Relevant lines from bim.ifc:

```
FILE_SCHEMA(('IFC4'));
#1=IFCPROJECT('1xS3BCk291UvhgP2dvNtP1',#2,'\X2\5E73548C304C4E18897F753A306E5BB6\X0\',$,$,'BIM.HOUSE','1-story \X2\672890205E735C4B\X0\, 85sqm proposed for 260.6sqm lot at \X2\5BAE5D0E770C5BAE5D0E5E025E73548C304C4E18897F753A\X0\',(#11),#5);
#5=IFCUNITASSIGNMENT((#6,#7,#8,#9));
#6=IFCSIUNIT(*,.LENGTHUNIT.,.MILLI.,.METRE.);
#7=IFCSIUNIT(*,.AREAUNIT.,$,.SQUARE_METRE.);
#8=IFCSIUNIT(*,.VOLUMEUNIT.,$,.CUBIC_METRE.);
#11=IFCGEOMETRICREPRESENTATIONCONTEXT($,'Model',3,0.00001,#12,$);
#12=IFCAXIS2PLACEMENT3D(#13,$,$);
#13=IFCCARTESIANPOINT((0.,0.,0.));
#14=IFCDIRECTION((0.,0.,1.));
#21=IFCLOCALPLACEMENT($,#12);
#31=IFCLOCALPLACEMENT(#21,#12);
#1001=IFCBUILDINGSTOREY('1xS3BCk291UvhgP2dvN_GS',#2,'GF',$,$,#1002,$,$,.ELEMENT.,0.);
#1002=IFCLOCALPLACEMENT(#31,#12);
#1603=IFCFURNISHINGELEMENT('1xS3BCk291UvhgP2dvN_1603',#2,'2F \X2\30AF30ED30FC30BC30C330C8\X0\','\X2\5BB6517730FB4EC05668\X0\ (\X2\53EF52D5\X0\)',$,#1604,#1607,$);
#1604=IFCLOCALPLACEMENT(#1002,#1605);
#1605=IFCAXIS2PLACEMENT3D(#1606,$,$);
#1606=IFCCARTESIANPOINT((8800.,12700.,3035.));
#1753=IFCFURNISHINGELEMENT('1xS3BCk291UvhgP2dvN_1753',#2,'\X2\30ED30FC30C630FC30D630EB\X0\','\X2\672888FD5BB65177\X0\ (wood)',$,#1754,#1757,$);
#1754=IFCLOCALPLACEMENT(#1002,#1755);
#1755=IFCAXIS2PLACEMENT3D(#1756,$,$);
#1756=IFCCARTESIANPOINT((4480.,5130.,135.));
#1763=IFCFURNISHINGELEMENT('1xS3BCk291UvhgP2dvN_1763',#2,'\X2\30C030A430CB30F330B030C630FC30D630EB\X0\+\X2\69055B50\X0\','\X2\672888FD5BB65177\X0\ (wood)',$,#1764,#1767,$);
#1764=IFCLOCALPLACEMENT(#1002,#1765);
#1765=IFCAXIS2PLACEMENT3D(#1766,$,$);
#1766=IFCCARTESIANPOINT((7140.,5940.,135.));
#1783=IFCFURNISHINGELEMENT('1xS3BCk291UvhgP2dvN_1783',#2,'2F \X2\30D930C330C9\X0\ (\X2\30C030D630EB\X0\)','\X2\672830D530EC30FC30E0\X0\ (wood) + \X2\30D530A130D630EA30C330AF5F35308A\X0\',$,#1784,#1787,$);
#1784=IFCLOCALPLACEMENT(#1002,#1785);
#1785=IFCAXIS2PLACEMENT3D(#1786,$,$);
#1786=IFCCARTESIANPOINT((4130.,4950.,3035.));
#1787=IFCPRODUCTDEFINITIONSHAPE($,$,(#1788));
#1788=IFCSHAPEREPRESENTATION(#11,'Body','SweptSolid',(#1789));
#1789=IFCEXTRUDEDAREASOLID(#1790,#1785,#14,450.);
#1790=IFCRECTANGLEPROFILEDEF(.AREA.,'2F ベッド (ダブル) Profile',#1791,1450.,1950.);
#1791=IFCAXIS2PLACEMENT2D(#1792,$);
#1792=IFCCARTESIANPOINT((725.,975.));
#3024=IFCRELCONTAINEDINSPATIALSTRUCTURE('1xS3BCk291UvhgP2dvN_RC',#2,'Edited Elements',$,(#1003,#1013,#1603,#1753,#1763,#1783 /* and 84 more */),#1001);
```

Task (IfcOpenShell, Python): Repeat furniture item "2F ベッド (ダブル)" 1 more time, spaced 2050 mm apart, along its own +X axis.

```python
import ifcopenshell
import ifcopenshell.api.geometry
import ifcopenshell.api.root
import ifcopenshell.util.element
import ifcopenshell.util.placement
import ifcopenshell.util.unit

model = ifcopenshell.open("bim.ifc")
unit_scale = ifcopenshell.util.unit.calculate_unit_scale(model)


def reuse_history(source, copy):
    """copy_class also copies each property set's owner history, people and application; keep the originals."""
    for rel in copy.IsDefinedBy:
        if rel.is_a("IfcRelDefinesByProperties") and (history := rel.RelatingPropertyDefinition.OwnerHistory):
            rel.RelatingPropertyDefinition.OwnerHistory = source.OwnerHistory
            ifcopenshell.util.element.remove_deep2(model, history)


source = model.by_guid("1xS3BCk291UvhgP2dvN_1783")
base = ifcopenshell.util.placement.get_local_placement(source.ObjectPlacement)
step = base[:3, 0] * 2.05 / unit_scale

for i in range(1, 2):
    copy = ifcopenshell.api.root.copy_class(model, product=source)
    copy.Representation = ifcopenshell.util.element.copy_deep(
        model, source.Representation, exclude=["IfcGeometricRepresentationContext", "IfcRepresentationMap"]
    )
    reuse_history(source, copy)
    matrix = base.copy()
    matrix[:3, 3] += i * step
    print("added at", matrix[:3, 3].round(3) + 0.0)
    ifcopenshell.api.geometry.edit_object_placement(model, product=copy, matrix=matrix, is_si=False)

model.write("bim_edited.ifc")
```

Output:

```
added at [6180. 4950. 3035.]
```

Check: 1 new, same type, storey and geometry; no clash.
